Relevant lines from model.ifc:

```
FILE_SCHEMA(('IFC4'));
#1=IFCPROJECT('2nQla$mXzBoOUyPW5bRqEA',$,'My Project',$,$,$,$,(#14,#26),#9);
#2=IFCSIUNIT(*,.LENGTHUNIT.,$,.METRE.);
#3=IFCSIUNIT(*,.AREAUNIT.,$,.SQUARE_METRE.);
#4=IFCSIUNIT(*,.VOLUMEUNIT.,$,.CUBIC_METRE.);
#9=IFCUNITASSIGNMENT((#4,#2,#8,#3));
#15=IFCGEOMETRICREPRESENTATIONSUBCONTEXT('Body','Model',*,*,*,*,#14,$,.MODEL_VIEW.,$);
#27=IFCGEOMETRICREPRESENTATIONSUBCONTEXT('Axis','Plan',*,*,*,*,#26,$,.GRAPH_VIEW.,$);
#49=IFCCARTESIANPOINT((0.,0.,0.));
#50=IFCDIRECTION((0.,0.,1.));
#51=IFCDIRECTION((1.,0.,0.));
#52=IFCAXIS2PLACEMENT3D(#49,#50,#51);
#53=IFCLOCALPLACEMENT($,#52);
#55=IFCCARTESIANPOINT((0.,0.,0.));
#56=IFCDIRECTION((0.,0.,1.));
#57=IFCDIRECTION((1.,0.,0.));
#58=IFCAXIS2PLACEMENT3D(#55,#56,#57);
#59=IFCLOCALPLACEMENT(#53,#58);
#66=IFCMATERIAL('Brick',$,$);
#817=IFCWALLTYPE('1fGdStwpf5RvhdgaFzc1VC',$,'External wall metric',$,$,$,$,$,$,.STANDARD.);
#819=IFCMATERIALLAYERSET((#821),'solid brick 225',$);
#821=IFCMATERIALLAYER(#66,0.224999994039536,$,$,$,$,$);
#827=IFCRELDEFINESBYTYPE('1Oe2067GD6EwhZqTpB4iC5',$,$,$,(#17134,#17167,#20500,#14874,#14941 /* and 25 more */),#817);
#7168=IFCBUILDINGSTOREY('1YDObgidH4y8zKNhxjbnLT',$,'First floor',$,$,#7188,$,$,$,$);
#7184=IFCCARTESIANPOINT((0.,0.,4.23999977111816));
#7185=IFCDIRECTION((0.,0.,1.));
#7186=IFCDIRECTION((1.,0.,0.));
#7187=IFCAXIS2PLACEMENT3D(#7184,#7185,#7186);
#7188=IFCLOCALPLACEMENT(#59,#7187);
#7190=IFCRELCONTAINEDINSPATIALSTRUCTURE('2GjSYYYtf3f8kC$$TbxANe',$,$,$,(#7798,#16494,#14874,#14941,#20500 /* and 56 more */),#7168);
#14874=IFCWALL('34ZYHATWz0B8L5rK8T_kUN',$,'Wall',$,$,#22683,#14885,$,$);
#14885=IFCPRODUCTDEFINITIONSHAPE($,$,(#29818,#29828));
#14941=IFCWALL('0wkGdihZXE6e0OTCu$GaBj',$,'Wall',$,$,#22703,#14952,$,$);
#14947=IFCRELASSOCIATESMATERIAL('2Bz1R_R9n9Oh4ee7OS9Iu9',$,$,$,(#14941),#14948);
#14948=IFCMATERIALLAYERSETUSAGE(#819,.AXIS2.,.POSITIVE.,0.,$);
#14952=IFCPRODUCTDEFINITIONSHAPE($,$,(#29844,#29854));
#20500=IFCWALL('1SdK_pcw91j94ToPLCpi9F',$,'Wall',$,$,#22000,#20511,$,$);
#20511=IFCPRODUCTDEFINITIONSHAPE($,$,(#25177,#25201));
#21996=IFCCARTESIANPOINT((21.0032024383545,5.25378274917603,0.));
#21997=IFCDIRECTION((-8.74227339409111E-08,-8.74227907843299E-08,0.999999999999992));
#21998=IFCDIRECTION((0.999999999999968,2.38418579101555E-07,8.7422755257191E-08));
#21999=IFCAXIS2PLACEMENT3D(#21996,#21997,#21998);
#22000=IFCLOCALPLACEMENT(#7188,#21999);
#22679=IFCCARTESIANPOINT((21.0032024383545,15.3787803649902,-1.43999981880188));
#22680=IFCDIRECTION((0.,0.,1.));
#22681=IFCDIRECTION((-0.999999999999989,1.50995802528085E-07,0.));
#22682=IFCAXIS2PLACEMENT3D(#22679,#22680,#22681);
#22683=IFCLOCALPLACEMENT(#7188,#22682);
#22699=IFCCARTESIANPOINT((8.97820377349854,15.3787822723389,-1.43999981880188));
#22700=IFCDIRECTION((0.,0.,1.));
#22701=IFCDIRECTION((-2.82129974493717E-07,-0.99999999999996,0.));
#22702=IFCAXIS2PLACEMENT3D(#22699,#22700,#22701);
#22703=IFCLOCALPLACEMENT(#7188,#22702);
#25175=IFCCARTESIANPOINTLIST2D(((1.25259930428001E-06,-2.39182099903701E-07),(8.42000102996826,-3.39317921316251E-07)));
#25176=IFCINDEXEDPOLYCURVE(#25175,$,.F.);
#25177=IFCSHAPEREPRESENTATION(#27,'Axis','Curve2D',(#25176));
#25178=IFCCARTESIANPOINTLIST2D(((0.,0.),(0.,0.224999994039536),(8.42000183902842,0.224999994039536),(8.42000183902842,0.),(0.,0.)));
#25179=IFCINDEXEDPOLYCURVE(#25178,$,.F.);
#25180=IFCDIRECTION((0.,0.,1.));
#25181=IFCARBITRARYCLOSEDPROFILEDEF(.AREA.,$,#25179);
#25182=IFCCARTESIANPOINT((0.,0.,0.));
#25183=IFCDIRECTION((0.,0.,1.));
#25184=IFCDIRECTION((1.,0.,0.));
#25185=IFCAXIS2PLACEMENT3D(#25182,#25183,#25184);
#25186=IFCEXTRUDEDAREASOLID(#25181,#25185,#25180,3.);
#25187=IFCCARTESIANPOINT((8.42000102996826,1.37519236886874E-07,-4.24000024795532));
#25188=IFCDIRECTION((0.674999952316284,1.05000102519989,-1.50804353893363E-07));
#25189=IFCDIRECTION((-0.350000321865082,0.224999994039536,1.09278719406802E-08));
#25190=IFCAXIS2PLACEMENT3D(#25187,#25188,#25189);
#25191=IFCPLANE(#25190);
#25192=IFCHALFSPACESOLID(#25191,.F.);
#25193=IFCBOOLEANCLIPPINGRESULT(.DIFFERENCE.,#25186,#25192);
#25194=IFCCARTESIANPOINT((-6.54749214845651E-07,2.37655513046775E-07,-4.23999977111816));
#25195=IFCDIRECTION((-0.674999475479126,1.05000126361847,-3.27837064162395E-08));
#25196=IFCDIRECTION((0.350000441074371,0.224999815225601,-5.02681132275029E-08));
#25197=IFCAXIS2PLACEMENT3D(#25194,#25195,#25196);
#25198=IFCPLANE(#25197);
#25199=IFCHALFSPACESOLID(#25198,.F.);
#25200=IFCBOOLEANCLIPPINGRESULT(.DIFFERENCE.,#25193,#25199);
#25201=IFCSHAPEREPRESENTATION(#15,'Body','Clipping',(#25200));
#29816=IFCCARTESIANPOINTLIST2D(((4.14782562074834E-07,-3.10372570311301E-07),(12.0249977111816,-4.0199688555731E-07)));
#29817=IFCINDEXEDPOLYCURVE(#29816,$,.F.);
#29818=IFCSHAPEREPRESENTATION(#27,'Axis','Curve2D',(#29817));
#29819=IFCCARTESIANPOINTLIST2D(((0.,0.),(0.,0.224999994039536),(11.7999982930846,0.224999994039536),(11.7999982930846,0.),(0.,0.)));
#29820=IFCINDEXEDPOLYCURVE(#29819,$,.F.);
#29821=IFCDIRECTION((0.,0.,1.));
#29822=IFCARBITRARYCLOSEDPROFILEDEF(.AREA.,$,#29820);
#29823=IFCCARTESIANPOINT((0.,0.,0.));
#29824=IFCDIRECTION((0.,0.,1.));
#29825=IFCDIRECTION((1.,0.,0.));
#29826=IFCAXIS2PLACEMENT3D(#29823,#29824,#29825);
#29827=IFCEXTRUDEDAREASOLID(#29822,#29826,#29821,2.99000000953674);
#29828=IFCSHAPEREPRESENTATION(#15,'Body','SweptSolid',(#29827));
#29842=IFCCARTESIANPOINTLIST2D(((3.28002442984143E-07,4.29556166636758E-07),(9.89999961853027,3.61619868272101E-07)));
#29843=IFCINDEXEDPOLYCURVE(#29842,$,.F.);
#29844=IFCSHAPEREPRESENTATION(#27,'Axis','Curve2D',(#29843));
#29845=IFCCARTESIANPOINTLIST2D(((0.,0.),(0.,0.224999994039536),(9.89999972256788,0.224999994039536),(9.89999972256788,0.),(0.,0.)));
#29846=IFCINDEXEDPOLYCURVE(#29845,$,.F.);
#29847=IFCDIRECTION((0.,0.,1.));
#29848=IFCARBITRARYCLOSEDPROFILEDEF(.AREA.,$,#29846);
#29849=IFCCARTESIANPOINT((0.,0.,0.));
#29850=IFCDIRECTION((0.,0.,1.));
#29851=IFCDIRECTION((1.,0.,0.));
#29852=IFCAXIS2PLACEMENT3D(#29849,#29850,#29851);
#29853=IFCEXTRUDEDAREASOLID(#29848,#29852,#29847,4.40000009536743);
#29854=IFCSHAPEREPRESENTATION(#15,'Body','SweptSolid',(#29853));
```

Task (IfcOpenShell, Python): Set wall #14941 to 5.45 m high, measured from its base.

```python
import ifcopenshell
import ifcopenshell.geom
import ifcopenshell.util.representation
import ifcopenshell.util.shape
import ifcopenshell.util.unit

model = ifcopenshell.open("model.ifc")
unit_scale = ifcopenshell.util.unit.calculate_unit_scale(model)
settings = ifcopenshell.geom.settings()


def volume(element):
    """Net volume in cubic metres, openings subtracted."""
    shape = ifcopenshell.geom.create_shape(settings, element)
    return ifcopenshell.util.shape.get_volume(shape.geometry)


wall = model.by_guid("0wkGdihZXE6e0OTCu$GaBj")
before = volume(wall)

body = ifcopenshell.util.representation.get_representation(wall, "Model", "Body")
solid = body.Items[0]
old_height = solid.Depth
solid.Depth = 5.45 / unit_scale
after = volume(wall)

print(f"height {old_height:g} -> {solid.Depth:g}, volume {before:.3f} -> {after:.3f} m3")

model.write("model_v2.ifc")
```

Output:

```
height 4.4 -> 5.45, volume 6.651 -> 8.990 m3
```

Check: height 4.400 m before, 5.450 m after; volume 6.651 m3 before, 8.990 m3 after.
